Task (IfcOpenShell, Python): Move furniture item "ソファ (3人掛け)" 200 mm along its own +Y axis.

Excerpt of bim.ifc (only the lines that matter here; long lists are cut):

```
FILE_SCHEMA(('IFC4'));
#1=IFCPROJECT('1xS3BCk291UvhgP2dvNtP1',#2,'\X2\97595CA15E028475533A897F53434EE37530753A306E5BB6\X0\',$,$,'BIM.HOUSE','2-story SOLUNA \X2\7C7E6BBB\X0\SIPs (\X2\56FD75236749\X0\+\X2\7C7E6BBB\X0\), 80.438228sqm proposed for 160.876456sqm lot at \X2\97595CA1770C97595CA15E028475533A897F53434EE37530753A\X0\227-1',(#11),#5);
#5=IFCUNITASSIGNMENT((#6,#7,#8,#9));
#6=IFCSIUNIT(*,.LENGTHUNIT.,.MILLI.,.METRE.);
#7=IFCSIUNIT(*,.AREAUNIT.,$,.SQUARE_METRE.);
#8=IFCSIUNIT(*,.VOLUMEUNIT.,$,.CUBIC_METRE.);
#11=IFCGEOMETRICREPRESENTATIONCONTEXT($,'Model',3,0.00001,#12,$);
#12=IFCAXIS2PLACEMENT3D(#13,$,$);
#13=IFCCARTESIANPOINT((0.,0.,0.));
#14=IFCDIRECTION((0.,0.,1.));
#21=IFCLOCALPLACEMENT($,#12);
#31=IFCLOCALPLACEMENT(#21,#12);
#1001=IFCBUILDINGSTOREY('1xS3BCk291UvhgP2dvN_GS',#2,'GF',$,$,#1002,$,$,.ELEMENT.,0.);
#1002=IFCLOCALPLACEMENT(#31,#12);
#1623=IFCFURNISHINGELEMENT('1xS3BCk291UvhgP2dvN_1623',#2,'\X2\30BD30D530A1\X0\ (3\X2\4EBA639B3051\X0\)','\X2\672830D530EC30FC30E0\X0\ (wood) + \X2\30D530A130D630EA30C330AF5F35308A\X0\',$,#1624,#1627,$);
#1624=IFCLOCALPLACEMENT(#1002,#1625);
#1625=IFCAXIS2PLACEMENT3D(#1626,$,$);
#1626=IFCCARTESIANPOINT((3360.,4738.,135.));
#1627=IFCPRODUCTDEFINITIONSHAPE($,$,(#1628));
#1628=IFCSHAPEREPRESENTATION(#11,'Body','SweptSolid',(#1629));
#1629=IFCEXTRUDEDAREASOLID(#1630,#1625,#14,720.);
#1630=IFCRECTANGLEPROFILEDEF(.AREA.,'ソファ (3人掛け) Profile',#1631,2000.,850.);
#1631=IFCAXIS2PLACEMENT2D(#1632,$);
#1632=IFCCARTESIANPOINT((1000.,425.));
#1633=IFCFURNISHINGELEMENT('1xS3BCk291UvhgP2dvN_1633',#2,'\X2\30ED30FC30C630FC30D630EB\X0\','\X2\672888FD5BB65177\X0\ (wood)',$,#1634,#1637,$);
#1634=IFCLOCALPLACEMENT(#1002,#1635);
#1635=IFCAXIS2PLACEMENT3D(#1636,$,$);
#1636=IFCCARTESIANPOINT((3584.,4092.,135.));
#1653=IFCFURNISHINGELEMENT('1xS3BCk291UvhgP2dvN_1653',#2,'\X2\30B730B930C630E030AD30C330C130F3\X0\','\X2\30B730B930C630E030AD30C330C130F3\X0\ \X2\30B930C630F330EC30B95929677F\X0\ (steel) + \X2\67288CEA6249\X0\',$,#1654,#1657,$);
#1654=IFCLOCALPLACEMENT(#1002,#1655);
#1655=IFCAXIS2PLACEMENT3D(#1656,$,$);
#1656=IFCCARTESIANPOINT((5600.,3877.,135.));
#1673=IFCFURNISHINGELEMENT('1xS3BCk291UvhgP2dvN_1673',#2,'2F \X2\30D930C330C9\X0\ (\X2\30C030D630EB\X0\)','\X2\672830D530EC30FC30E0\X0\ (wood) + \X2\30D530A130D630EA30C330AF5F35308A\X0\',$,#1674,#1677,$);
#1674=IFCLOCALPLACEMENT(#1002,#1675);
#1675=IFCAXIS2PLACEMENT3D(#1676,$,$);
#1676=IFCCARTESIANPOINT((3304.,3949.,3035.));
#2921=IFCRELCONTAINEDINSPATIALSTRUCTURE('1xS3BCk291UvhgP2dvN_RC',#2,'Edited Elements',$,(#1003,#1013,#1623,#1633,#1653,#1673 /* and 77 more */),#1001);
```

```python
import ifcopenshell
import ifcopenshell.api.geometry
import ifcopenshell.util.placement
import ifcopenshell.util.unit

model = ifcopenshell.open("bim.ifc")
unit_scale = ifcopenshell.util.unit.calculate_unit_scale(model)

item = model.by_guid("1xS3BCk291UvhgP2dvN_1623")
matrix = ifcopenshell.util.placement.get_local_placement(item.ObjectPlacement)
matrix[:3, 3] += matrix[:3, 1] * 0.2 / unit_scale
ifcopenshell.api.geometry.edit_object_placement(model, product=item, matrix=matrix, is_si=False)

print(ifcopenshell.util.placement.get_local_placement(item.ObjectPlacement).round(3) + 0.0)

model.write("bim_v2.ifc")
```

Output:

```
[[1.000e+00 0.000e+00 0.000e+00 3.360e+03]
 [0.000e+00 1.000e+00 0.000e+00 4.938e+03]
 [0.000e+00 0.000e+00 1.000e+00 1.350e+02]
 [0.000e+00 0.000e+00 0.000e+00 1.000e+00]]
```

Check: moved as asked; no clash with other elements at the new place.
